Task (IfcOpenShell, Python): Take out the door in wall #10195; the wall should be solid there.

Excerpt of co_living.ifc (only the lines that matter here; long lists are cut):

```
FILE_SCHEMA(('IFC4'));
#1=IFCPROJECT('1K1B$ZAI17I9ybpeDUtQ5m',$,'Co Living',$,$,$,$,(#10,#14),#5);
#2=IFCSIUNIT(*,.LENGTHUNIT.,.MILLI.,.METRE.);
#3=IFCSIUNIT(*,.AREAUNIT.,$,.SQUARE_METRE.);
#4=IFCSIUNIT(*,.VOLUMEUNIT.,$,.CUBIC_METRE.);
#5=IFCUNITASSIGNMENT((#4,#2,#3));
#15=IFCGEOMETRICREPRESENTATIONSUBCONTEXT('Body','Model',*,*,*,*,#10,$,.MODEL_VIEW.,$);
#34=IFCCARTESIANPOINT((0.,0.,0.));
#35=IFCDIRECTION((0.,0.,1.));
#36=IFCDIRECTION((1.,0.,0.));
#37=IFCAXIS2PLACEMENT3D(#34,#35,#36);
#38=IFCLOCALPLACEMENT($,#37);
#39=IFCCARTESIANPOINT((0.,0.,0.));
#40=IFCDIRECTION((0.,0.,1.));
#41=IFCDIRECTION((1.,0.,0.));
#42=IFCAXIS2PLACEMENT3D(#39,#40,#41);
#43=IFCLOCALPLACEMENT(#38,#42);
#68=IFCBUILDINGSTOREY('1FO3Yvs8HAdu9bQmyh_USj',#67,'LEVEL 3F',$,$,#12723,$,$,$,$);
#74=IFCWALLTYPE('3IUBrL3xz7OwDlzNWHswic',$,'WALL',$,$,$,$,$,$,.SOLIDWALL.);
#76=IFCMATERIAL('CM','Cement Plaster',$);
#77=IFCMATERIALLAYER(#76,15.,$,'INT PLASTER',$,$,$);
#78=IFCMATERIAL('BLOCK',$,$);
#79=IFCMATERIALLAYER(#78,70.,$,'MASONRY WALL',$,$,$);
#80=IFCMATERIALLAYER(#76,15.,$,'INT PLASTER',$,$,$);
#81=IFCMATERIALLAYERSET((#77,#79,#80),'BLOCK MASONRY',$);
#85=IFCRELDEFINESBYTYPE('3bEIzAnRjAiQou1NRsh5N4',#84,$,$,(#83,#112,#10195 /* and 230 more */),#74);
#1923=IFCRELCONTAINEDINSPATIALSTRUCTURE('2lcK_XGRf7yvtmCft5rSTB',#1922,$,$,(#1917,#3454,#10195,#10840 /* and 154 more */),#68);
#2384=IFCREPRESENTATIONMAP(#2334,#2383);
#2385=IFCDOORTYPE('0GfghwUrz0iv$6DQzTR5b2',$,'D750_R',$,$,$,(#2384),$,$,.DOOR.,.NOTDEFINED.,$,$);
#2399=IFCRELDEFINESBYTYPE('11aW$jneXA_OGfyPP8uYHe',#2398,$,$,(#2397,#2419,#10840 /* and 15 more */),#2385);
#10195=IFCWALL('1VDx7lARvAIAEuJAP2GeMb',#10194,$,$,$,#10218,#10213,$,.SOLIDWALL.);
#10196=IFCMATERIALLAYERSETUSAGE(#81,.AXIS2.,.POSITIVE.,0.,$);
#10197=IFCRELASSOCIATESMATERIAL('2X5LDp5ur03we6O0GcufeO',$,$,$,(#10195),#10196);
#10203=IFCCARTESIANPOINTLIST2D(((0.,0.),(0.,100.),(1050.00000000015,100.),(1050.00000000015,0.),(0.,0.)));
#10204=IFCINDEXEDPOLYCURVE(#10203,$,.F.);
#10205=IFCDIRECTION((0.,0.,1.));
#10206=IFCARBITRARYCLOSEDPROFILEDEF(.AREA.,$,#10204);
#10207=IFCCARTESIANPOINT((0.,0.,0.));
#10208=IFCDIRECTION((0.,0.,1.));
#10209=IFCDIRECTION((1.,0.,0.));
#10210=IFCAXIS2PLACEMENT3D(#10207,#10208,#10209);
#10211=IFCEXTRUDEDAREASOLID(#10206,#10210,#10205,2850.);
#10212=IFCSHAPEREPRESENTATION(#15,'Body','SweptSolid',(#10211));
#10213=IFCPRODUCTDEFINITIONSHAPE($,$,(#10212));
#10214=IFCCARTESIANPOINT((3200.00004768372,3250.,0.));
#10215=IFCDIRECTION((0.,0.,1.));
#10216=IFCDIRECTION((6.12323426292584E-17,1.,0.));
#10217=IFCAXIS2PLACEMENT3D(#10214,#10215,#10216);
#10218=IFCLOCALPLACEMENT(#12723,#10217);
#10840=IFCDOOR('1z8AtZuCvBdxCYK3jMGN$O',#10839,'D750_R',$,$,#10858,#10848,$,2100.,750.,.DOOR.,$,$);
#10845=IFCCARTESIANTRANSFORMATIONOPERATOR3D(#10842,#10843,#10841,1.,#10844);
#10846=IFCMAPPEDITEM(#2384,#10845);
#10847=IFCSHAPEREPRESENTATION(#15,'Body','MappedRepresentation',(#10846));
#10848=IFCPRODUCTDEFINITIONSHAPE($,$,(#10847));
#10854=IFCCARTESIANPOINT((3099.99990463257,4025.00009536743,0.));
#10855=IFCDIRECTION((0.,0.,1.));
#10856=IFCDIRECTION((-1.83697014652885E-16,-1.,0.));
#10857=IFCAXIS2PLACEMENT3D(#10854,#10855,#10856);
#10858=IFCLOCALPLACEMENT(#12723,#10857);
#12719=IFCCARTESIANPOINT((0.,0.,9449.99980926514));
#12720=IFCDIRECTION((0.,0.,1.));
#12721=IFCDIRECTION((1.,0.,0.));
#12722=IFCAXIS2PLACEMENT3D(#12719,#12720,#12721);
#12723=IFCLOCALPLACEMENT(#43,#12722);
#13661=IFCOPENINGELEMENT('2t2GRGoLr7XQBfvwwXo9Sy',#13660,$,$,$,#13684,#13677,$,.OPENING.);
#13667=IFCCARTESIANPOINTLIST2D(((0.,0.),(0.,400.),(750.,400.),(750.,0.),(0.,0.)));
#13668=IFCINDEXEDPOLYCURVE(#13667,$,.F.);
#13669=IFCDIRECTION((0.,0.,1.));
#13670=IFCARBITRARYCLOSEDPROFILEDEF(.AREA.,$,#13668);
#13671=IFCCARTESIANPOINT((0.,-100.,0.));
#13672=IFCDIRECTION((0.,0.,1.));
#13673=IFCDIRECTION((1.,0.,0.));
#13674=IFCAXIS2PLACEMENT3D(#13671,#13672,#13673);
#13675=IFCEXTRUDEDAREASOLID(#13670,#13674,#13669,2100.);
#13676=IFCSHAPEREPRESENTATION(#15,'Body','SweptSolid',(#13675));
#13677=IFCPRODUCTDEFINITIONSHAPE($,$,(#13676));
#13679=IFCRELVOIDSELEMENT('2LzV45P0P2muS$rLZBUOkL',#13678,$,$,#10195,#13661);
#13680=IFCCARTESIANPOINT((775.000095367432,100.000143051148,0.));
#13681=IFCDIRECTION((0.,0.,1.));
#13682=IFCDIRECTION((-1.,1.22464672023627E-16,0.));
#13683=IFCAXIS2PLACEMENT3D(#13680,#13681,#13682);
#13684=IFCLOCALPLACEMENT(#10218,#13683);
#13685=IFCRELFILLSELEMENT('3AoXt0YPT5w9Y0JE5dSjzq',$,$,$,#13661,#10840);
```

```python
import ifcopenshell
import ifcopenshell.api.feature
import ifcopenshell.api.root
import ifcopenshell.geom
import ifcopenshell.util.shape

model = ifcopenshell.open("co_living.ifc")
settings = ifcopenshell.geom.settings()


def volume(element):
    """Net volume in cubic metres, openings subtracted."""
    shape = ifcopenshell.geom.create_shape(settings, element)
    return ifcopenshell.util.shape.get_volume(shape.geometry)


door = model.by_id(10840)
opening = door.FillsVoids[0].RelatingOpeningElement
wall = opening.VoidsElements[0].RelatingBuildingElement
before = volume(wall)

ifcopenshell.api.root.remove_product(model, product=door)
ifcopenshell.api.feature.remove_feature(model, feature=opening)

after = volume(wall)

print(f"wall volume {before:.3f} -> {after:.3f} m3")

model.write("co_living-out.ifc")
```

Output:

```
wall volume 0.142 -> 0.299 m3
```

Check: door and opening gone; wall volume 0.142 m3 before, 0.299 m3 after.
